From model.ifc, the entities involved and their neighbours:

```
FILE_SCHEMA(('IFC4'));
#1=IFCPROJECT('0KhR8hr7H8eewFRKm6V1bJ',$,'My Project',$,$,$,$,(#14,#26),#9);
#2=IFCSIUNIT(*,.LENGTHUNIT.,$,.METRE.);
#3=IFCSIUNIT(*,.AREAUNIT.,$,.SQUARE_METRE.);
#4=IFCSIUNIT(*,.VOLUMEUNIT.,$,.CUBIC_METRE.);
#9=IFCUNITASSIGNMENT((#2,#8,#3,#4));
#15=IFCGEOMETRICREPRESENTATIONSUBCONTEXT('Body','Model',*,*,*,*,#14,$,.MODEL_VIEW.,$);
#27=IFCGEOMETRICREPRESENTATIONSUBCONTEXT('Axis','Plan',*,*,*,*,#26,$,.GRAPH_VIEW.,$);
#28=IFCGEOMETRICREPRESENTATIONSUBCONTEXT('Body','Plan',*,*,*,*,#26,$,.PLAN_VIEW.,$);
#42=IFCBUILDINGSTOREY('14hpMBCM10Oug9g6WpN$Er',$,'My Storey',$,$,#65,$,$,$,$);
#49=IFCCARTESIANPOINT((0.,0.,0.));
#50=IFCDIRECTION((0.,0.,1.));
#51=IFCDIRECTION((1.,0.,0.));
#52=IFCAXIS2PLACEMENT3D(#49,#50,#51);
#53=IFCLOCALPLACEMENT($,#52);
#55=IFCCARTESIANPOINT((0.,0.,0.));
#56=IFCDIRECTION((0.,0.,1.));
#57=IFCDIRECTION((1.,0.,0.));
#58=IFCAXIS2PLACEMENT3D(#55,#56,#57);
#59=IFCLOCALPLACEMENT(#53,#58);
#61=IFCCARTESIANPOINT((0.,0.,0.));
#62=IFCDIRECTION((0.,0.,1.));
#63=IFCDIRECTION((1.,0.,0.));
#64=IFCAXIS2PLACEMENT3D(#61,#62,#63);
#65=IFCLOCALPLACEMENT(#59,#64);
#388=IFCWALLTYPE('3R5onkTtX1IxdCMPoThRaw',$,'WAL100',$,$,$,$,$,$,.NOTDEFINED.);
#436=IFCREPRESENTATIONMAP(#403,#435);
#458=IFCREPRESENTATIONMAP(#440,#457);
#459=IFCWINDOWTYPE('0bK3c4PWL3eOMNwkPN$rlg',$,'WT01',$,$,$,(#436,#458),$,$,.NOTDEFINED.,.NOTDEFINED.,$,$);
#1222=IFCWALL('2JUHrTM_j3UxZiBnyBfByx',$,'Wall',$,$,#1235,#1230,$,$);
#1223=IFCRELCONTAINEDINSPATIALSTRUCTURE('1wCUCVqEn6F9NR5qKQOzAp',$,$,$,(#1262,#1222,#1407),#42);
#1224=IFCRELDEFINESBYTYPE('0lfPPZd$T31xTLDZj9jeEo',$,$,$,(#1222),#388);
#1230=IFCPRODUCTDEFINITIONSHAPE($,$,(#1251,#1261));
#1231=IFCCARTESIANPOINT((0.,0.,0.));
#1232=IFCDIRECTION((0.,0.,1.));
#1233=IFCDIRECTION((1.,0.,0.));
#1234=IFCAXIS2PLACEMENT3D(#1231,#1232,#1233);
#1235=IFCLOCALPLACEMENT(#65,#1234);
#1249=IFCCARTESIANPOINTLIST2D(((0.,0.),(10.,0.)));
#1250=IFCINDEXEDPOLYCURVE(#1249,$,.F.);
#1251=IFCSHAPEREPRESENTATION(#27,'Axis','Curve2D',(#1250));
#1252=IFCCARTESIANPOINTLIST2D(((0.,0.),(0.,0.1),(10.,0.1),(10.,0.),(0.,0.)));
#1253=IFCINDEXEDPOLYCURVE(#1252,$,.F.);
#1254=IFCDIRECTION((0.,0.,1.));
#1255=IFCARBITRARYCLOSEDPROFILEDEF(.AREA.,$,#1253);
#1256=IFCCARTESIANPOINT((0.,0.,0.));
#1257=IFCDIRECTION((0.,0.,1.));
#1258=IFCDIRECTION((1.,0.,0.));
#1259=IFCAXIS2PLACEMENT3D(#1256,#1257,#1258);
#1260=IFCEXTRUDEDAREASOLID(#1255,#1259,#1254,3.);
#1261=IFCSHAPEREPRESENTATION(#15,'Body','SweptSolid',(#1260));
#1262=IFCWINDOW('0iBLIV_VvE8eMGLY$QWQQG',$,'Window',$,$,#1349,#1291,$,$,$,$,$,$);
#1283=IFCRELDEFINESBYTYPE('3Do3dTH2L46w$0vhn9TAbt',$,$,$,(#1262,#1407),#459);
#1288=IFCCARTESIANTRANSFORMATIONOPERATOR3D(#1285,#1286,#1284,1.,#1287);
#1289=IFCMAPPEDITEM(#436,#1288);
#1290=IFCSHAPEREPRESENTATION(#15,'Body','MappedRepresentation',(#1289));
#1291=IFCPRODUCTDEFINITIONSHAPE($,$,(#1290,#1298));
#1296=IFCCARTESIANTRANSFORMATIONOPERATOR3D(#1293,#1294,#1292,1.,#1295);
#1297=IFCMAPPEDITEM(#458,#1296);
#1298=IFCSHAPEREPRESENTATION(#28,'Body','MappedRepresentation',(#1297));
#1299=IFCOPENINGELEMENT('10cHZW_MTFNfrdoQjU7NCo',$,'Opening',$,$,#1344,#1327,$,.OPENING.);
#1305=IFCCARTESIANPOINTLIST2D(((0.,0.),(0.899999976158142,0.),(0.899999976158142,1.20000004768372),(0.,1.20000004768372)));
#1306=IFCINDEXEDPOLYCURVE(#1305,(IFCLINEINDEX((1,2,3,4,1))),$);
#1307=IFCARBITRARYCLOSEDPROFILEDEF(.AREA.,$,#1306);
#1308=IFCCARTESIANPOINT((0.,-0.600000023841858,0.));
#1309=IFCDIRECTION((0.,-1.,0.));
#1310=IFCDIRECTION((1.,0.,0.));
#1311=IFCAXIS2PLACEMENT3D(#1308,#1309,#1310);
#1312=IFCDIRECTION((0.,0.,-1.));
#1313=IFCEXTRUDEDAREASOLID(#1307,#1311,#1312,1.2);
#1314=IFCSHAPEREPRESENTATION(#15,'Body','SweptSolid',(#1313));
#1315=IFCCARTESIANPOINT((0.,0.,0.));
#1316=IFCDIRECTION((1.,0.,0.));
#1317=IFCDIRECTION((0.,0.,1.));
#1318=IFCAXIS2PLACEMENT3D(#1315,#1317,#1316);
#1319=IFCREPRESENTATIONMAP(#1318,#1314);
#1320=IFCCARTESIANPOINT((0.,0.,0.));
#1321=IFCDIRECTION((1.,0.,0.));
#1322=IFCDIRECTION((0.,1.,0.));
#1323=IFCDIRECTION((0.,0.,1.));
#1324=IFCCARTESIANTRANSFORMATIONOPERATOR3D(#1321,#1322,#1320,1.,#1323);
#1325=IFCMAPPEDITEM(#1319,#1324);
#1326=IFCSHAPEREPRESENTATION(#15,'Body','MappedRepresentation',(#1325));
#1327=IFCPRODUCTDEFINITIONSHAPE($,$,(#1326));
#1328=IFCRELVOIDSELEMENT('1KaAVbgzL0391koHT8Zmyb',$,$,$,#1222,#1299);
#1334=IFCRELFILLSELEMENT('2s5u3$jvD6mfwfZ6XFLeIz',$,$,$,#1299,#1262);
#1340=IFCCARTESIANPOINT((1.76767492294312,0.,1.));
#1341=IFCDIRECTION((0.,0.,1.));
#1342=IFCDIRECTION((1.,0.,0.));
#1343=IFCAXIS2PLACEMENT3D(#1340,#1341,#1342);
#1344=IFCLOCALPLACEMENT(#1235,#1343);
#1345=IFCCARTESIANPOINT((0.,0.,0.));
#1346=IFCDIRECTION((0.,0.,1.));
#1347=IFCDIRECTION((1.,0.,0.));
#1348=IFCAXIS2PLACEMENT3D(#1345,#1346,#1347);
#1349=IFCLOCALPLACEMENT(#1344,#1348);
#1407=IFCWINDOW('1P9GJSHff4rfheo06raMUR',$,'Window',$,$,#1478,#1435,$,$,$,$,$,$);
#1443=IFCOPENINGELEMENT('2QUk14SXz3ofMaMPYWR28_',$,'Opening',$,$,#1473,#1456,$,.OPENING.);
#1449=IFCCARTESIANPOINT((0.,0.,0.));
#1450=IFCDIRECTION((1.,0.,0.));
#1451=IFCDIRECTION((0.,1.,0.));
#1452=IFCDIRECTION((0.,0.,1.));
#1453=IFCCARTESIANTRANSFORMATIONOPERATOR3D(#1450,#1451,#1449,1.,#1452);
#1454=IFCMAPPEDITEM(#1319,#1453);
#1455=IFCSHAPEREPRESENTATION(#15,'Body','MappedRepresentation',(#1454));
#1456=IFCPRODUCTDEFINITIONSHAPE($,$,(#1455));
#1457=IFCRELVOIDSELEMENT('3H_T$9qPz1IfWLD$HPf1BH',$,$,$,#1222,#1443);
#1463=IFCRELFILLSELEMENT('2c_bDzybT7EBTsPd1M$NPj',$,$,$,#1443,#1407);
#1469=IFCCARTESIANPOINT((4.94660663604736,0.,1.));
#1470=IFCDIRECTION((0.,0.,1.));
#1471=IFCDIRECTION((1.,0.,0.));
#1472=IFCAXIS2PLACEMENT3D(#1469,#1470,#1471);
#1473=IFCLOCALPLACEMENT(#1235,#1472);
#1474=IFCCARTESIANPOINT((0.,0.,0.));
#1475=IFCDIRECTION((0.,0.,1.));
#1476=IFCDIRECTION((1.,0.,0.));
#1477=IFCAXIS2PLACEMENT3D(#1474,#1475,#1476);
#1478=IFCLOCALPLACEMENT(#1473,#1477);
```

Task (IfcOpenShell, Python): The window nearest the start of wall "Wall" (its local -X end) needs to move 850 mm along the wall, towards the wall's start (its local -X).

```python
import ifcopenshell
import ifcopenshell.api.geometry
import ifcopenshell.util.placement

model = ifcopenshell.open("model.ifc")

window = model.by_guid("0iBLIV_VvE8eMGLY$QWQQG")
opening = window.FillsVoids[0].RelatingOpeningElement
wall = opening.VoidsElements[0].RelatingBuildingElement

wall_matrix = ifcopenshell.util.placement.get_local_placement(wall.ObjectPlacement)
shift = wall_matrix[:3, 0] * -0.85
before = ifcopenshell.util.placement.get_local_placement(window.ObjectPlacement)[:3, 3].copy()

# The window is placed relative to its opening, so it follows when the opening moves.
matrix = ifcopenshell.util.placement.get_local_placement(opening.ObjectPlacement)
matrix[:3, 3] += shift
ifcopenshell.api.geometry.edit_object_placement(
    model, product=opening, matrix=matrix, is_si=False, should_transform_children=True
)

after = ifcopenshell.util.placement.get_local_placement(window.ObjectPlacement)[:3, 3]
print("window moved by", (after - before).round(3) + 0.0)

model.write("model_updated.ifc")
```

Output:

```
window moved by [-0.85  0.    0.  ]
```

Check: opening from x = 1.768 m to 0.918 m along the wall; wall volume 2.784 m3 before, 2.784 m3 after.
